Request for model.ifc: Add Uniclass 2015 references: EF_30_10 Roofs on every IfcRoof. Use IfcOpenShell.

First a look at what the model holds.

```python
import ifcopenshell

model = ifcopenshell.open("model.ifc")
print(model.schema)
print("classifications:", [c.Name for c in model.by_type("IfcClassification")])
for ifc_class in ("IfcDoor", "IfcRoof", "IfcStair", "IfcWall", "IfcWindow"):
    print(ifc_class, len(model.by_type(ifc_class)))
```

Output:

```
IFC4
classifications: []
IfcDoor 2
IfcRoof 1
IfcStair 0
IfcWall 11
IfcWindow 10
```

```python
import ifcopenshell
import ifcopenshell.api.classification

model = ifcopenshell.open("model.ifc")

system = ifcopenshell.api.classification.add_classification(model, classification="Uniclass 2015")

codes = {
    "IfcRoof": ("EF_30_10", "Roofs"),
}
for ifc_class, (code, name) in codes.items():
    products = model.by_type(ifc_class)
    ifcopenshell.api.classification.add_reference(
        model, products=products, classification=system, identification=code, name=name
    )
    print(code, len(products))

model.write("model-out.ifc")
```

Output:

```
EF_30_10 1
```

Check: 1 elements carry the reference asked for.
